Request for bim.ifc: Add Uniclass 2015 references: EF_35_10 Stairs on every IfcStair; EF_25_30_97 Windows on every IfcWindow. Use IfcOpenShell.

First a look at what the model holds.

```python
import ifcopenshell

model = ifcopenshell.open("bim.ifc")
print(model.schema)
print("classifications:", [c.Name for c in model.by_type("IfcClassification")])
for ifc_class in ("IfcDoor", "IfcRoof", "IfcStair", "IfcWall", "IfcWindow"):
    print(ifc_class, len(model.by_type(ifc_class)))
```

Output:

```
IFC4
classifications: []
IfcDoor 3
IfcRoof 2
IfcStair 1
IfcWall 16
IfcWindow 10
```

```python
import ifcopenshell
import ifcopenshell.api.classification

model = ifcopenshell.open("bim.ifc")

system = ifcopenshell.api.classification.add_classification(model, classification="Uniclass 2015")

codes = {
    "IfcStair": ("EF_35_10", "Stairs"),
    "IfcWindow": ("EF_25_30_97", "Windows"),
}
for ifc_class, (code, name) in codes.items():
    products = model.by_type(ifc_class)
    ifcopenshell.api.classification.add_reference(
        model, products=products, classification=system, identification=code, name=name
    )
    print(code, len(products))

model.write("bim-out.ifc")
```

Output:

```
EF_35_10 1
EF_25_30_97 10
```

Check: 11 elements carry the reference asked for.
